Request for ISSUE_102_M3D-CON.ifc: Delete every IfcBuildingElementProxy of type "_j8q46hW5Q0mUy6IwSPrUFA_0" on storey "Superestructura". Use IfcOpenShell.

First a look at what the model holds.

```python
import ifcopenshell
import ifcopenshell.util.element

model = ifcopenshell.open("ISSUE_102_M3D-CON.ifc")
print(model.schema)
storey = next(s for s in model.by_type("IfcBuildingStorey") if s.Name == "Superestructura")
proxies = [e for e in ifcopenshell.util.element.get_decomposition(storey) if e.is_a("IfcBuildingElementProxy")]
seen = {}
for e in proxies:
    element_type = ifcopenshell.util.element.get_type(e)
    name = element_type.Name if element_type not in (None, e) else None
    seen[name] = seen.get(name, 0) + 1
for name, count in sorted(seen.items(), key=str):
    print(count, "x", name)
```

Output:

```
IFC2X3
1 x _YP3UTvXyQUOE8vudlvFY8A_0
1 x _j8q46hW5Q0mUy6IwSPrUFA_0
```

```python
import ifcopenshell
import ifcopenshell.api.root
import ifcopenshell.util.element

model = ifcopenshell.open("ISSUE_102_M3D-CON.ifc")

storey = next(s for s in model.by_type("IfcBuildingStorey") if s.Name == "Superestructura")
proxies = [e for e in ifcopenshell.util.element.get_decomposition(storey) if e.is_a("IfcBuildingElementProxy")]
targets = [e for e in proxies if (t := ifcopenshell.util.element.get_type(e)) not in (None, e) and t.Name == "_j8q46hW5Q0mUy6IwSPrUFA_0"]

for e in targets:
    ifcopenshell.api.root.remove_product(model, product=e)
print(len(targets), "removed")

model.write("ISSUE_102_M3D-CON_rev.ifc")
```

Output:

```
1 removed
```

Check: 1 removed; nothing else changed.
